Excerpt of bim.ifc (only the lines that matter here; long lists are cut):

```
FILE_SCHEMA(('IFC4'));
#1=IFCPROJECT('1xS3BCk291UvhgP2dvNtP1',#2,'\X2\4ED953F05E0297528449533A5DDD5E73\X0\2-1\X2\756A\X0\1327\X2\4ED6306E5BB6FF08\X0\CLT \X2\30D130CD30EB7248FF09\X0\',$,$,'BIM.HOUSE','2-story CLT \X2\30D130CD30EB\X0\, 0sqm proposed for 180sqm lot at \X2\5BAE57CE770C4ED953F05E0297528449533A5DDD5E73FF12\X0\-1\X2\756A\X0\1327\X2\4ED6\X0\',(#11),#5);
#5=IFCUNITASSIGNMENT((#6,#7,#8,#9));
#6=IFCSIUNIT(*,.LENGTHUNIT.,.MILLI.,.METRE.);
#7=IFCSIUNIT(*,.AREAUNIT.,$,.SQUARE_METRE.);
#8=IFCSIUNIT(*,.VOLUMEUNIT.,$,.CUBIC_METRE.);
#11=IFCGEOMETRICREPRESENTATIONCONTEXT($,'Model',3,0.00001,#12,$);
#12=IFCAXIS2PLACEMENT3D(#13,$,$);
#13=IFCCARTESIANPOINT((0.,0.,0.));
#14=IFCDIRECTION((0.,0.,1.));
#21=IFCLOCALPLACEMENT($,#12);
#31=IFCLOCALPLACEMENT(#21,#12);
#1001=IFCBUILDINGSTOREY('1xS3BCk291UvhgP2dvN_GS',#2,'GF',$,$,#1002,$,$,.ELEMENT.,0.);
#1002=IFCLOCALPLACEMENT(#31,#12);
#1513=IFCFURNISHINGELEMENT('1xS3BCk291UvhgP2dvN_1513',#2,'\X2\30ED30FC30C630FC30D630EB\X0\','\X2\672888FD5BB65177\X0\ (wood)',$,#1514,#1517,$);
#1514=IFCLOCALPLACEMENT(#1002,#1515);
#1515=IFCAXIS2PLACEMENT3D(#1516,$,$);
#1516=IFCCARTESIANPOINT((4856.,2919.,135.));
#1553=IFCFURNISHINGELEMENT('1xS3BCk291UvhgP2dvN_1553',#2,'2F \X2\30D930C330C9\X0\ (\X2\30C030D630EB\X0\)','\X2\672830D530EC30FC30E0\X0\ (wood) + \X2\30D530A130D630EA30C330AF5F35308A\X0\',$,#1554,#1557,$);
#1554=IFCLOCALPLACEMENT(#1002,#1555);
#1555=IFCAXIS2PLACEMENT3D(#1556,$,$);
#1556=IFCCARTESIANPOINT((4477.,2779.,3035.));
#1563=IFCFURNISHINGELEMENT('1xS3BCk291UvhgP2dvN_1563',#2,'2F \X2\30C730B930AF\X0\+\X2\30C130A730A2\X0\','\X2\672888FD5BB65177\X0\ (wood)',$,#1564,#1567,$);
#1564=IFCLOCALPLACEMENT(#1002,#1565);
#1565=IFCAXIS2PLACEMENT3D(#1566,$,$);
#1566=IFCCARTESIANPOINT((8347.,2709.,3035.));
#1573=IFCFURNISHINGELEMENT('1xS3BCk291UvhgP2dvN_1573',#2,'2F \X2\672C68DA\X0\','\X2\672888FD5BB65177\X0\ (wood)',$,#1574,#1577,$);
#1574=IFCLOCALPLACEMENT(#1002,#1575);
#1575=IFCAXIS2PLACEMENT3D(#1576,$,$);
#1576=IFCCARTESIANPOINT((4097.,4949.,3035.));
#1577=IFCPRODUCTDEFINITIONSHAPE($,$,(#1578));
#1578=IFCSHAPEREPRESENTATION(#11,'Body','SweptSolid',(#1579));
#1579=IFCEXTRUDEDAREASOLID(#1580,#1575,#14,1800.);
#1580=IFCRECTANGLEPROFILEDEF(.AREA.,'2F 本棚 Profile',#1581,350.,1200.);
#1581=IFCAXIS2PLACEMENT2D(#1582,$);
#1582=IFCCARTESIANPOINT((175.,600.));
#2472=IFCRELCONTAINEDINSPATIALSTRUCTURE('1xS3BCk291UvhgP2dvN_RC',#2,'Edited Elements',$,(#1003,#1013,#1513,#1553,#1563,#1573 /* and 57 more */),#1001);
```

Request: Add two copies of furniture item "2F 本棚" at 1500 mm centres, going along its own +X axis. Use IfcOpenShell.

```python
import ifcopenshell
import ifcopenshell.api.geometry
import ifcopenshell.api.root
import ifcopenshell.util.element
import ifcopenshell.util.placement

model = ifcopenshell.open("bim.ifc")


def reuse_history(source, copy):
    """copy_class also copies each property set's owner history, people and application; keep the originals."""
    for rel in copy.IsDefinedBy:
        if rel.is_a("IfcRelDefinesByProperties") and (history := rel.RelatingPropertyDefinition.OwnerHistory):
            rel.RelatingPropertyDefinition.OwnerHistory = source.OwnerHistory
            ifcopenshell.util.element.remove_deep2(model, history)


source = model.by_guid("1xS3BCk291UvhgP2dvN_1573")
base = ifcopenshell.util.placement.get_local_placement(source.ObjectPlacement)
step = base[:3, 0] * 1500.0

for i in range(1, 3):
    copy = ifcopenshell.api.root.copy_class(model, product=source)
    copy.Representation = ifcopenshell.util.element.copy_deep(
        model, source.Representation, exclude=["IfcGeometricRepresentationContext", "IfcRepresentationMap"]
    )
    reuse_history(source, copy)
    matrix = base.copy()
    matrix[:3, 3] += i * step
    print("added at", matrix[:3, 3].round(3) + 0.0)
    ifcopenshell.api.geometry.edit_object_placement(model, product=copy, matrix=matrix, is_si=False)

model.write("bim_v2.ifc")
```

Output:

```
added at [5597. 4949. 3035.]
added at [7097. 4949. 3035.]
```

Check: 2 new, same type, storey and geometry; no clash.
